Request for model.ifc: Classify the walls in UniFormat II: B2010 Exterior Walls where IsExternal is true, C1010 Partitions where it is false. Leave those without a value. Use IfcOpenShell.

First a look at what the model holds.

```python
import ifcopenshell
import ifcopenshell.util.element

model = ifcopenshell.open("model.ifc")
print(model.schema)
print("classifications:", [c.Name for c in model.by_type("IfcClassification")])
values = [ifcopenshell.util.element.get_pset(e, "Pset_WallCommon", "IsExternal") for e in model.by_type("IfcWall")]
for value in (True, False, None):
    print("IsExternal", value, values.count(value))
```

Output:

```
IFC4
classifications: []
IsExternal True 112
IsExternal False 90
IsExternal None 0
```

```python
import ifcopenshell
import ifcopenshell.api.classification
import ifcopenshell.util.element

model = ifcopenshell.open("model.ifc")

system = ifcopenshell.api.classification.add_classification(model, classification="UniFormat II")

walls = model.by_type("IfcWall")
external = {e: ifcopenshell.util.element.get_pset(e, "Pset_WallCommon", "IsExternal") for e in walls}
for flag, code, name in ((True, "B2010", "Exterior Walls"), (False, "C1010", "Partitions")):
    products = [e for e in walls if external[e] is flag]
    ifcopenshell.api.classification.add_reference(
        model, products=products, classification=system, identification=code, name=name
    )
    print(code, len(products))

model.write("model_updated.ifc")
```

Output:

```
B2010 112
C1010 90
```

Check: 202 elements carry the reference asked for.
